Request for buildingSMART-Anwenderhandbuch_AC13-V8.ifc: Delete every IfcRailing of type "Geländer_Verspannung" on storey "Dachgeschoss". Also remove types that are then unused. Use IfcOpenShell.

First a look at what the model holds.

```python
import ifcopenshell
import ifcopenshell.util.element

model = ifcopenshell.open("buildingSMART-Anwenderhandbuch_AC13-V8.ifc")
print(model.schema)
storey = next(s for s in model.by_type("IfcBuildingStorey") if s.Name == "Dachgeschoss")
railings = [e for e in ifcopenshell.util.element.get_decomposition(storey) if e.is_a("IfcRailing")]
seen = {}
for e in railings:
    element_type = ifcopenshell.util.element.get_type(e)
    name = element_type.Name if element_type not in (None, e) else None
    seen[name] = seen.get(name, 0) + 1
for name, count in sorted(seen.items(), key=str):
    print(count, "x", name)
```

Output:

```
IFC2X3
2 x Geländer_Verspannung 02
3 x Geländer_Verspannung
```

```python
import ifcopenshell
import ifcopenshell.api.root
import ifcopenshell.util.element

model = ifcopenshell.open("buildingSMART-Anwenderhandbuch_AC13-V8.ifc")

storey = next(s for s in model.by_type("IfcBuildingStorey") if s.Name == "Dachgeschoss")
railings = [e for e in ifcopenshell.util.element.get_decomposition(storey) if e.is_a("IfcRailing")]
targets = [e for e in railings if (t := ifcopenshell.util.element.get_type(e)) not in (None, e) and t.Name == "Geländer_Verspannung"]
types = {ifcopenshell.util.element.get_type(e) for e in targets} - {None, *targets}

for e in targets:
    ifcopenshell.api.root.remove_product(model, product=e)
print(len(targets), "removed")

unused = [t for t in types if not ifcopenshell.util.element.get_types(t)]
for t in unused:
    ifcopenshell.api.root.remove_product(model, product=t)
print(len(unused), "unused types removed")

model.write("buildingSMART-Anwenderhandbuch_AC13-V8-out.ifc")
```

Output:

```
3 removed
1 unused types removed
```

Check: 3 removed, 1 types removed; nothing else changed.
